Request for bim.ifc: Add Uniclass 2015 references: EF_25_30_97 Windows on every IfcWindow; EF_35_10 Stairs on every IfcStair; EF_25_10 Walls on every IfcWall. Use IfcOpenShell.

First a look at what the model holds.

```python
import ifcopenshell

model = ifcopenshell.open("bim.ifc")
print(model.schema)
print("classifications:", [c.Name for c in model.by_type("IfcClassification")])
for ifc_class in ("IfcDoor", "IfcRoof", "IfcStair", "IfcWall", "IfcWindow"):
    print(ifc_class, len(model.by_type(ifc_class)))
```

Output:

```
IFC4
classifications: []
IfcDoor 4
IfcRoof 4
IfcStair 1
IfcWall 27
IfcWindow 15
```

```python
import ifcopenshell
import ifcopenshell.api.classification

model = ifcopenshell.open("bim.ifc")

system = ifcopenshell.api.classification.add_classification(model, classification="Uniclass 2015")

codes = {
    "IfcWindow": ("EF_25_30_97", "Windows"),
    "IfcStair": ("EF_35_10", "Stairs"),
    "IfcWall": ("EF_25_10", "Walls"),
}
for ifc_class, (code, name) in codes.items():
    products = model.by_type(ifc_class)
    ifcopenshell.api.classification.add_reference(
        model, products=products, classification=system, identification=code, name=name
    )
    print(code, len(products))

model.write("bim_updated.ifc")
```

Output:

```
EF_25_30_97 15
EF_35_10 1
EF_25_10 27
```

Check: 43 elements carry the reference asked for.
